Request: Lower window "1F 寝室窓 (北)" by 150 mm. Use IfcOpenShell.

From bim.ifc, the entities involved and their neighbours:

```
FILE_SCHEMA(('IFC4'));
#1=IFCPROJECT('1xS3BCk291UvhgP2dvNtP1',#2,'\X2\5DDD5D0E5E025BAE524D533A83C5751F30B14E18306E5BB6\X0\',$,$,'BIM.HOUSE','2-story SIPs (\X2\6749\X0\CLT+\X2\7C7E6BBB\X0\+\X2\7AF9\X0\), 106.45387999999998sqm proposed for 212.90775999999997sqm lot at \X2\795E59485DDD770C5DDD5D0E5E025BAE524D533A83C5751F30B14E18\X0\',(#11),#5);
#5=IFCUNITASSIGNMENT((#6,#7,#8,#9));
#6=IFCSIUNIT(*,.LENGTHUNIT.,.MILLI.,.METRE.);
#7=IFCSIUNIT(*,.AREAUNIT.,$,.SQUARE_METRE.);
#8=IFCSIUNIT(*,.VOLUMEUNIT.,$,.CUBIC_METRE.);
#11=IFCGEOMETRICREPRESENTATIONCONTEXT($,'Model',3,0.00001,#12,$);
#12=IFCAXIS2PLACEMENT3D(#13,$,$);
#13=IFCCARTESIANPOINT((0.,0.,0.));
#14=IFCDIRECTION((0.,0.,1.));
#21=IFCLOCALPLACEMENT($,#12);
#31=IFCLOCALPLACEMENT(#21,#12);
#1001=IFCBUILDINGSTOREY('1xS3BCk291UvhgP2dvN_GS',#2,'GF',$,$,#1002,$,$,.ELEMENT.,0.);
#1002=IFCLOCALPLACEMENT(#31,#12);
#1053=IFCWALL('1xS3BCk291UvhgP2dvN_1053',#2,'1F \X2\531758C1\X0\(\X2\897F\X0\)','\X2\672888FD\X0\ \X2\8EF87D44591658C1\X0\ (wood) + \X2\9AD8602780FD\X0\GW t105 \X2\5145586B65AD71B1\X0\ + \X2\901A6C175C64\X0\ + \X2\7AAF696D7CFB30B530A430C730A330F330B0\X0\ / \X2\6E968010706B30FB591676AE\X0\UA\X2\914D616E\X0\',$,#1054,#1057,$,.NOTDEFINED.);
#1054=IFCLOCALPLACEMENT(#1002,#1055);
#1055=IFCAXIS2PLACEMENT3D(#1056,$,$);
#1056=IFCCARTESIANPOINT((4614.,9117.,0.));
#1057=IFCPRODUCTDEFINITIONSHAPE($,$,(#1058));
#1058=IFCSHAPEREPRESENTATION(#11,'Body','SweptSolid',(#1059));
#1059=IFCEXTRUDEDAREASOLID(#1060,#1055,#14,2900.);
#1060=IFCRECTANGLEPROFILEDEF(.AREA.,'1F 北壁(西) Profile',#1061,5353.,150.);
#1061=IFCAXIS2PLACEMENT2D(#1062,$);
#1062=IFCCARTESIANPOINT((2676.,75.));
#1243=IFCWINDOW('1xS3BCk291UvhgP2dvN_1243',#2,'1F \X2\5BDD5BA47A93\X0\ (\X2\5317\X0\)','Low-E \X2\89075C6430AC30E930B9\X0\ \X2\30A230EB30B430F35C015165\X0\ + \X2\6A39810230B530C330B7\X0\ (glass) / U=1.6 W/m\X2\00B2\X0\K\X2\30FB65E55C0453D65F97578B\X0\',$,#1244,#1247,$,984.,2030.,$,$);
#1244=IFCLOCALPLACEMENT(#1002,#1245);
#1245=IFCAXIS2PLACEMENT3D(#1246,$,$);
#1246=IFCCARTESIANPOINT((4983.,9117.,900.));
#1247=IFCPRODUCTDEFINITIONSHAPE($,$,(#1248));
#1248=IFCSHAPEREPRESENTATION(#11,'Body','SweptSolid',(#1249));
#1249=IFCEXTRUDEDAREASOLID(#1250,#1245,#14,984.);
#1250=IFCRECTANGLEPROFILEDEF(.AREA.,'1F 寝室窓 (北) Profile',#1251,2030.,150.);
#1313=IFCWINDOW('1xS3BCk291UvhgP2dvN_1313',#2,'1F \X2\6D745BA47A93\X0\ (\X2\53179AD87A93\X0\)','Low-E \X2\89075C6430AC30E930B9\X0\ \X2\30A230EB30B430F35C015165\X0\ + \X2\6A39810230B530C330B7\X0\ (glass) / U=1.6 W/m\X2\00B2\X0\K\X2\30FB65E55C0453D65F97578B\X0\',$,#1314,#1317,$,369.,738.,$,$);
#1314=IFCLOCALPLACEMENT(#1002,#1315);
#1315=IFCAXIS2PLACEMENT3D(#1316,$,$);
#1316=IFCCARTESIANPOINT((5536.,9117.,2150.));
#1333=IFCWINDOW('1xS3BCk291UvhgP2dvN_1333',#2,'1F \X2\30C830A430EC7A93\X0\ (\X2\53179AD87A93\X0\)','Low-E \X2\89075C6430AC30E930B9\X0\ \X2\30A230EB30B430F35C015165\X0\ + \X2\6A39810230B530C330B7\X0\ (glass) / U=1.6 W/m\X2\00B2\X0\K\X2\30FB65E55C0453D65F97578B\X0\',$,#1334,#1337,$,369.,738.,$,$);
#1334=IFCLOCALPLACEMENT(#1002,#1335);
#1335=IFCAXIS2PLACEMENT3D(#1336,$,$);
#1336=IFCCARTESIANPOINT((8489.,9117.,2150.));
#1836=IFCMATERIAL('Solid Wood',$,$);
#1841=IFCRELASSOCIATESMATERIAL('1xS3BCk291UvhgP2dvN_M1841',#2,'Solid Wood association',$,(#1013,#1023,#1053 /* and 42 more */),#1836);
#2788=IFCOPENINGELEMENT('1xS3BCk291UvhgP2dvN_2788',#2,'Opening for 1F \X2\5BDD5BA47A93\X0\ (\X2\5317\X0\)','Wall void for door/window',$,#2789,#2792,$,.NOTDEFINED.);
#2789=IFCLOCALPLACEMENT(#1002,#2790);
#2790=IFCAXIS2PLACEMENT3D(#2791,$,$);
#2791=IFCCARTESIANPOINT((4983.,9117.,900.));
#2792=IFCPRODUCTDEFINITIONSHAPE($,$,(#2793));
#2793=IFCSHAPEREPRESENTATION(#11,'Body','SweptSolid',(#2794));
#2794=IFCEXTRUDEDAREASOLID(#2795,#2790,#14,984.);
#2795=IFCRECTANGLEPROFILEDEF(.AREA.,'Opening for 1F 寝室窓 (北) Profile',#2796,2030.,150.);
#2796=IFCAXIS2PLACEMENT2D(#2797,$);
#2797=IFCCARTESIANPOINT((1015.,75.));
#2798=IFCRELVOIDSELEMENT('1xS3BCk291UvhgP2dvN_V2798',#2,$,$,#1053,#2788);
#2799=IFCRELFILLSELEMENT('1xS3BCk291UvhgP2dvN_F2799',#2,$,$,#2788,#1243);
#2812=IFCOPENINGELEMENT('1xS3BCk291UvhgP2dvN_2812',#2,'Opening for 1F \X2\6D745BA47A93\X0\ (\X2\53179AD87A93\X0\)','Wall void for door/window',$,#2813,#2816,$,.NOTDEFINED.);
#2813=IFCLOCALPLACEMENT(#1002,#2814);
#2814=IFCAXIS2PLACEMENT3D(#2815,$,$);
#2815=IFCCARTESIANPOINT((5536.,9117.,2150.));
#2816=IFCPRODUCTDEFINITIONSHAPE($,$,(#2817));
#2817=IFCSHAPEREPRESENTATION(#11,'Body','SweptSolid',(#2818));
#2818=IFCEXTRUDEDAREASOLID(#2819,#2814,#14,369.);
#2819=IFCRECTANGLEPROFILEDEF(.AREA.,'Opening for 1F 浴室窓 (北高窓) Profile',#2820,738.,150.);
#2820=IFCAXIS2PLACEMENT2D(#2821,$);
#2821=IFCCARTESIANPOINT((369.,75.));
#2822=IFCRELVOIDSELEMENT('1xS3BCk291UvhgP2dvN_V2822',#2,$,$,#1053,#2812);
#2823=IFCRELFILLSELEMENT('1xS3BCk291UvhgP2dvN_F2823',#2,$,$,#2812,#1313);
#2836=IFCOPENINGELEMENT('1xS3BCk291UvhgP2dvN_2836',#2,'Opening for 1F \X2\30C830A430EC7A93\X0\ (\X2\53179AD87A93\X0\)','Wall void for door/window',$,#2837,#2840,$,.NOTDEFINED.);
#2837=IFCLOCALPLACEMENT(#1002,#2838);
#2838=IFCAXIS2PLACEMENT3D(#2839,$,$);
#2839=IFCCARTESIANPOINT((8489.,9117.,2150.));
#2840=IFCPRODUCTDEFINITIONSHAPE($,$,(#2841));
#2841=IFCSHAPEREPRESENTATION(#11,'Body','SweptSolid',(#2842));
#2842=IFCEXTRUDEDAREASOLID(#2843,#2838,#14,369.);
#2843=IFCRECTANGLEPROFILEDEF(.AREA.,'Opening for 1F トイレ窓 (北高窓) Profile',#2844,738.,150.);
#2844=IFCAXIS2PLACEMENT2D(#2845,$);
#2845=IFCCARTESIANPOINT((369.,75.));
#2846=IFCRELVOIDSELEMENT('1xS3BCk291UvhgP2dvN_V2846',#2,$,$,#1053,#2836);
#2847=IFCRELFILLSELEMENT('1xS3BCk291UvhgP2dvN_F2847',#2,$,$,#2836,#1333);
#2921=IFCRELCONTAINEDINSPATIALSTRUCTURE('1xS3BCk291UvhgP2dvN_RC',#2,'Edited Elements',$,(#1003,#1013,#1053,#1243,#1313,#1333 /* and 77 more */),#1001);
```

```python
import numpy as np
import ifcopenshell
import ifcopenshell.api.geometry
import ifcopenshell.util.placement
import ifcopenshell.util.unit

model = ifcopenshell.open("bim.ifc")
unit_scale = ifcopenshell.util.unit.calculate_unit_scale(model)

window = model.by_id(1243)
opening = window.FillsVoids[0].RelatingOpeningElement
dz = -0.15 / unit_scale

shift = np.array([0.0, 0.0, dz])
# The window is not placed relative to its opening, so move both.
for product in (opening, window):
    matrix = ifcopenshell.util.placement.get_local_placement(product.ObjectPlacement)
    matrix[:3, 3] += shift
    ifcopenshell.api.geometry.edit_object_placement(model, product=product, matrix=matrix, is_si=False)

print(f"moved by {dz * unit_scale:+.3f} m")

model.write("bim_v2.ifc")
```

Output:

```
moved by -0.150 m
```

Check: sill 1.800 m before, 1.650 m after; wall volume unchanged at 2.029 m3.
